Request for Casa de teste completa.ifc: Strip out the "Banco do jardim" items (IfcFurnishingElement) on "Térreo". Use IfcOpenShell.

First a look at what the model holds.

```python
import ifcopenshell
import ifcopenshell.util.element

model = ifcopenshell.open("Casa de teste completa.ifc")
print(model.schema)
storey = next(s for s in model.by_type("IfcBuildingStorey") if s.Name == "Térreo")
furniture = [e for e in ifcopenshell.util.element.get_decomposition(storey) if e.is_a("IfcFurnishingElement")]
seen = {}
for e in furniture:
    element_type = ifcopenshell.util.element.get_type(e)
    name = element_type.Name if element_type not in (None, e) else None
    seen[name] = seen.get(name, 0) + 1
for name, count in sorted(seen.items(), key=str):
    print(count, "x", name)
```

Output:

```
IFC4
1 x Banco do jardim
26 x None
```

```python
import ifcopenshell
import ifcopenshell.api.root
import ifcopenshell.util.element

model = ifcopenshell.open("Casa de teste completa.ifc")

storey = next(s for s in model.by_type("IfcBuildingStorey") if s.Name == "Térreo")
furniture = [e for e in ifcopenshell.util.element.get_decomposition(storey) if e.is_a("IfcFurnishingElement")]
targets = [e for e in furniture if (t := ifcopenshell.util.element.get_type(e)) not in (None, e) and t.Name == "Banco do jardim"]

for e in targets:
    ifcopenshell.api.root.remove_product(model, product=e)
print(len(targets), "removed")

model.write("Casa de teste completa_updated.ifc")
```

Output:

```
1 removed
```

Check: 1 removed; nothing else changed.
